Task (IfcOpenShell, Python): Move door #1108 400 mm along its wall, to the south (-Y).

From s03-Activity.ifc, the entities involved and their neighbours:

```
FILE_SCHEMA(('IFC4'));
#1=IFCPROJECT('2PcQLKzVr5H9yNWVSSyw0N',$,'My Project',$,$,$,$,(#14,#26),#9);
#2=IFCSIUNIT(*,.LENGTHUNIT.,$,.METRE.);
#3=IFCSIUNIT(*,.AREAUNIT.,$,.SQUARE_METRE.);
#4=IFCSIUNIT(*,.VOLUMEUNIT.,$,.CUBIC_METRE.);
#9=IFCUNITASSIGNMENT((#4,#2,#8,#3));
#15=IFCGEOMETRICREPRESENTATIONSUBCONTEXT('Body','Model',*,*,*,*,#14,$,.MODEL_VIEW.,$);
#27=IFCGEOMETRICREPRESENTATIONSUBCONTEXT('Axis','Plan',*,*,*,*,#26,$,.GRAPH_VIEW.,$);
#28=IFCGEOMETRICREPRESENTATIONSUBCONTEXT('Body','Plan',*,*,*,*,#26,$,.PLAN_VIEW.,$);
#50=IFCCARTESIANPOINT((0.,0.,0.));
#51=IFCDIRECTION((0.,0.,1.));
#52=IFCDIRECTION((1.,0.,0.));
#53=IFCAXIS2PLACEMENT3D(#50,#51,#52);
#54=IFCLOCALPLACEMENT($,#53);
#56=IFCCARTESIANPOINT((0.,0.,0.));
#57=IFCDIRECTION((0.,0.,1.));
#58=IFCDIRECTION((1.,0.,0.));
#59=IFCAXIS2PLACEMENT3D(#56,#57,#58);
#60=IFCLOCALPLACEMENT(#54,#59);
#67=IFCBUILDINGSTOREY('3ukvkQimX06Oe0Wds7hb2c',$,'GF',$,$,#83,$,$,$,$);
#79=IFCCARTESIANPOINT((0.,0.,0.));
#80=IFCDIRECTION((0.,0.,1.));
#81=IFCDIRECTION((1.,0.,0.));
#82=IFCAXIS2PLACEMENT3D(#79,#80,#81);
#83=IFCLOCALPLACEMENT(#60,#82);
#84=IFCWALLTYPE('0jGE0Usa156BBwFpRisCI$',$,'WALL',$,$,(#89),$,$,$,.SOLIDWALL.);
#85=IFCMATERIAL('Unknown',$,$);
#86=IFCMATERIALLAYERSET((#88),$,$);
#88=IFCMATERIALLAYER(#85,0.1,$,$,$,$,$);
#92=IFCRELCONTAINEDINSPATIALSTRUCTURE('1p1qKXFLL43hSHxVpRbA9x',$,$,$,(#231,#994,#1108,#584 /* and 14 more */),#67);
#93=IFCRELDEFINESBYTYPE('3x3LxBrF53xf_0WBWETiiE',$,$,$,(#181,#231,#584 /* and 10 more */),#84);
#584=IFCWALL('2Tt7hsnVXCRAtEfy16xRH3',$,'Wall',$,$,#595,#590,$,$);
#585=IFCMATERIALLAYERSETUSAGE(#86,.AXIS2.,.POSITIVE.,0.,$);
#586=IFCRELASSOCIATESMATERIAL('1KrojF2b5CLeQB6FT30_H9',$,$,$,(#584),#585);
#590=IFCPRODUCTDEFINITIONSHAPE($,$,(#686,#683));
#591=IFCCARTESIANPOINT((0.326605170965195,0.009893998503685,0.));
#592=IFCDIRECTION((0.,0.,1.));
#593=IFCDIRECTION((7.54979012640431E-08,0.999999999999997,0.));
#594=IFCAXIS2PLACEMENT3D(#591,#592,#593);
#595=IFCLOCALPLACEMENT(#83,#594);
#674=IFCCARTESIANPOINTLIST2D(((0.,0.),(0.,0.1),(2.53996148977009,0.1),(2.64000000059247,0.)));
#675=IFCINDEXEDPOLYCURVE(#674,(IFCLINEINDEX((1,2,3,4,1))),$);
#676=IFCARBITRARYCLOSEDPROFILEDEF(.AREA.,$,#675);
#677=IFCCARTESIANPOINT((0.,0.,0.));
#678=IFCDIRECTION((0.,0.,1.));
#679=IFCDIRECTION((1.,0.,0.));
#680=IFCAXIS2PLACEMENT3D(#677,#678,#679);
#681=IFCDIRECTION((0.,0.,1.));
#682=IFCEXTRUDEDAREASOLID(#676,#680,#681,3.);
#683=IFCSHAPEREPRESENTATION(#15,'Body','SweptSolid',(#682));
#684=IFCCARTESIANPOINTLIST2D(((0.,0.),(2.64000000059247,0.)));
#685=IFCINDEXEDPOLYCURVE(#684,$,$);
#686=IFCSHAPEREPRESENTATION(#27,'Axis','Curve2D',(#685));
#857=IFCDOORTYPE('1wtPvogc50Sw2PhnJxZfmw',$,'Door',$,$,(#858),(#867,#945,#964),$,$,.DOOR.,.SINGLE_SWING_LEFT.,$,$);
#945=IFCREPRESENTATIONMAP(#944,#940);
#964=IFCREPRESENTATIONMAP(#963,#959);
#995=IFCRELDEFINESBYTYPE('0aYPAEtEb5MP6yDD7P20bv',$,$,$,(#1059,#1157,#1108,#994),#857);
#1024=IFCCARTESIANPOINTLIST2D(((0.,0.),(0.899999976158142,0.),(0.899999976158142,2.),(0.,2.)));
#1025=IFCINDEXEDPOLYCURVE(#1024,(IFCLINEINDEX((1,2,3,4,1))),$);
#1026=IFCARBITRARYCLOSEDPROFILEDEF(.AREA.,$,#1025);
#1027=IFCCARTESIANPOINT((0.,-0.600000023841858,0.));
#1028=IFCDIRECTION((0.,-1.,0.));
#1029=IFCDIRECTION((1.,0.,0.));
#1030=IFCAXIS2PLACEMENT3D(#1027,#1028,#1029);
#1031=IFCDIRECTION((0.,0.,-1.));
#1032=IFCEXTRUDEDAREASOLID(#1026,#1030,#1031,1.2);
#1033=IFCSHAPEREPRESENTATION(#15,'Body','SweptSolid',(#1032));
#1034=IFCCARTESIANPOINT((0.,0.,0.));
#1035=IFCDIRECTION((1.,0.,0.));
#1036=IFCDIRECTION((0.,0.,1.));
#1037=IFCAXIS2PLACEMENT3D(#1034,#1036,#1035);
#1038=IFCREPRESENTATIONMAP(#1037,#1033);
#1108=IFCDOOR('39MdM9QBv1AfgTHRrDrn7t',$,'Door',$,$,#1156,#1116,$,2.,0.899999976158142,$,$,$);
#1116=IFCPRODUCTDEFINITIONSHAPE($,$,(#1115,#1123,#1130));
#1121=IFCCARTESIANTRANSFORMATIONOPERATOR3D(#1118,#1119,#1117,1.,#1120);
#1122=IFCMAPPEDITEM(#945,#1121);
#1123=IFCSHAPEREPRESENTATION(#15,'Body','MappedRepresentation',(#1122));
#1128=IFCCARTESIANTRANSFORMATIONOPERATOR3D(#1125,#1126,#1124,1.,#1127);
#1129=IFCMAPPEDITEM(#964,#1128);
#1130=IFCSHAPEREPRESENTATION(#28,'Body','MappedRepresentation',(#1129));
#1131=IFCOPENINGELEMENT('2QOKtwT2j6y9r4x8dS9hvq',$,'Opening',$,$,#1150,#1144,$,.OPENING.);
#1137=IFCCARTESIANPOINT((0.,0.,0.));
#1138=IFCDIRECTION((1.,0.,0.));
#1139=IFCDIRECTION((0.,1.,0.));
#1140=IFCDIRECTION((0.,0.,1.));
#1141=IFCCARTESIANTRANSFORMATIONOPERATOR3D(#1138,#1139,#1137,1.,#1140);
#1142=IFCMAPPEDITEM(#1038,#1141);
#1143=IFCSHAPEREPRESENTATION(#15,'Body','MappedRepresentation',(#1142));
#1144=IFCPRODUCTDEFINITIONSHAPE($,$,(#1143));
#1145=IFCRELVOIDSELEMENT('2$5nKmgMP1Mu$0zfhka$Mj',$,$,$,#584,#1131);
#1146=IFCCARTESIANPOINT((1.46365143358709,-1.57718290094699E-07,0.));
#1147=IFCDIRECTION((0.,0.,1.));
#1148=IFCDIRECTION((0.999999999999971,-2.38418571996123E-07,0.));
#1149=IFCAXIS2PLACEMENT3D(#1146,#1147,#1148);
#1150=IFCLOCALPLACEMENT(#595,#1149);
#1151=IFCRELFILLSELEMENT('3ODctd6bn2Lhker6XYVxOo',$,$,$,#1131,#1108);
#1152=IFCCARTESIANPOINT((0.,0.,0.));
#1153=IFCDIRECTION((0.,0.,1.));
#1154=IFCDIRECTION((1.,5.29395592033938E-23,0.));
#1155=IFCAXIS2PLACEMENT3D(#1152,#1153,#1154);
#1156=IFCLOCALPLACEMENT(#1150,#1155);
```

```python
import ifcopenshell
import ifcopenshell.api.geometry
import ifcopenshell.util.placement

model = ifcopenshell.open("s03-Activity.ifc")

door = model.by_id(1108)
opening = door.FillsVoids[0].RelatingOpeningElement
wall = opening.VoidsElements[0].RelatingBuildingElement

wall_matrix = ifcopenshell.util.placement.get_local_placement(wall.ObjectPlacement)
shift = wall_matrix[:3, 0] * -0.4
before = ifcopenshell.util.placement.get_local_placement(door.ObjectPlacement)[:3, 3].copy()

# The door is placed relative to its opening, so it follows when the opening moves.
matrix = ifcopenshell.util.placement.get_local_placement(opening.ObjectPlacement)
matrix[:3, 3] += shift
ifcopenshell.api.geometry.edit_object_placement(
    model, product=opening, matrix=matrix, is_si=False, should_transform_children=True
)

after = ifcopenshell.util.placement.get_local_placement(door.ObjectPlacement)[:3, 3]
print("door moved by", (after - before).round(3) + 0.0)

model.write("s03-Activity-out.ifc")
```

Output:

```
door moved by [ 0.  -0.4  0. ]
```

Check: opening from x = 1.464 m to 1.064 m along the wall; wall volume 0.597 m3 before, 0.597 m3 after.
